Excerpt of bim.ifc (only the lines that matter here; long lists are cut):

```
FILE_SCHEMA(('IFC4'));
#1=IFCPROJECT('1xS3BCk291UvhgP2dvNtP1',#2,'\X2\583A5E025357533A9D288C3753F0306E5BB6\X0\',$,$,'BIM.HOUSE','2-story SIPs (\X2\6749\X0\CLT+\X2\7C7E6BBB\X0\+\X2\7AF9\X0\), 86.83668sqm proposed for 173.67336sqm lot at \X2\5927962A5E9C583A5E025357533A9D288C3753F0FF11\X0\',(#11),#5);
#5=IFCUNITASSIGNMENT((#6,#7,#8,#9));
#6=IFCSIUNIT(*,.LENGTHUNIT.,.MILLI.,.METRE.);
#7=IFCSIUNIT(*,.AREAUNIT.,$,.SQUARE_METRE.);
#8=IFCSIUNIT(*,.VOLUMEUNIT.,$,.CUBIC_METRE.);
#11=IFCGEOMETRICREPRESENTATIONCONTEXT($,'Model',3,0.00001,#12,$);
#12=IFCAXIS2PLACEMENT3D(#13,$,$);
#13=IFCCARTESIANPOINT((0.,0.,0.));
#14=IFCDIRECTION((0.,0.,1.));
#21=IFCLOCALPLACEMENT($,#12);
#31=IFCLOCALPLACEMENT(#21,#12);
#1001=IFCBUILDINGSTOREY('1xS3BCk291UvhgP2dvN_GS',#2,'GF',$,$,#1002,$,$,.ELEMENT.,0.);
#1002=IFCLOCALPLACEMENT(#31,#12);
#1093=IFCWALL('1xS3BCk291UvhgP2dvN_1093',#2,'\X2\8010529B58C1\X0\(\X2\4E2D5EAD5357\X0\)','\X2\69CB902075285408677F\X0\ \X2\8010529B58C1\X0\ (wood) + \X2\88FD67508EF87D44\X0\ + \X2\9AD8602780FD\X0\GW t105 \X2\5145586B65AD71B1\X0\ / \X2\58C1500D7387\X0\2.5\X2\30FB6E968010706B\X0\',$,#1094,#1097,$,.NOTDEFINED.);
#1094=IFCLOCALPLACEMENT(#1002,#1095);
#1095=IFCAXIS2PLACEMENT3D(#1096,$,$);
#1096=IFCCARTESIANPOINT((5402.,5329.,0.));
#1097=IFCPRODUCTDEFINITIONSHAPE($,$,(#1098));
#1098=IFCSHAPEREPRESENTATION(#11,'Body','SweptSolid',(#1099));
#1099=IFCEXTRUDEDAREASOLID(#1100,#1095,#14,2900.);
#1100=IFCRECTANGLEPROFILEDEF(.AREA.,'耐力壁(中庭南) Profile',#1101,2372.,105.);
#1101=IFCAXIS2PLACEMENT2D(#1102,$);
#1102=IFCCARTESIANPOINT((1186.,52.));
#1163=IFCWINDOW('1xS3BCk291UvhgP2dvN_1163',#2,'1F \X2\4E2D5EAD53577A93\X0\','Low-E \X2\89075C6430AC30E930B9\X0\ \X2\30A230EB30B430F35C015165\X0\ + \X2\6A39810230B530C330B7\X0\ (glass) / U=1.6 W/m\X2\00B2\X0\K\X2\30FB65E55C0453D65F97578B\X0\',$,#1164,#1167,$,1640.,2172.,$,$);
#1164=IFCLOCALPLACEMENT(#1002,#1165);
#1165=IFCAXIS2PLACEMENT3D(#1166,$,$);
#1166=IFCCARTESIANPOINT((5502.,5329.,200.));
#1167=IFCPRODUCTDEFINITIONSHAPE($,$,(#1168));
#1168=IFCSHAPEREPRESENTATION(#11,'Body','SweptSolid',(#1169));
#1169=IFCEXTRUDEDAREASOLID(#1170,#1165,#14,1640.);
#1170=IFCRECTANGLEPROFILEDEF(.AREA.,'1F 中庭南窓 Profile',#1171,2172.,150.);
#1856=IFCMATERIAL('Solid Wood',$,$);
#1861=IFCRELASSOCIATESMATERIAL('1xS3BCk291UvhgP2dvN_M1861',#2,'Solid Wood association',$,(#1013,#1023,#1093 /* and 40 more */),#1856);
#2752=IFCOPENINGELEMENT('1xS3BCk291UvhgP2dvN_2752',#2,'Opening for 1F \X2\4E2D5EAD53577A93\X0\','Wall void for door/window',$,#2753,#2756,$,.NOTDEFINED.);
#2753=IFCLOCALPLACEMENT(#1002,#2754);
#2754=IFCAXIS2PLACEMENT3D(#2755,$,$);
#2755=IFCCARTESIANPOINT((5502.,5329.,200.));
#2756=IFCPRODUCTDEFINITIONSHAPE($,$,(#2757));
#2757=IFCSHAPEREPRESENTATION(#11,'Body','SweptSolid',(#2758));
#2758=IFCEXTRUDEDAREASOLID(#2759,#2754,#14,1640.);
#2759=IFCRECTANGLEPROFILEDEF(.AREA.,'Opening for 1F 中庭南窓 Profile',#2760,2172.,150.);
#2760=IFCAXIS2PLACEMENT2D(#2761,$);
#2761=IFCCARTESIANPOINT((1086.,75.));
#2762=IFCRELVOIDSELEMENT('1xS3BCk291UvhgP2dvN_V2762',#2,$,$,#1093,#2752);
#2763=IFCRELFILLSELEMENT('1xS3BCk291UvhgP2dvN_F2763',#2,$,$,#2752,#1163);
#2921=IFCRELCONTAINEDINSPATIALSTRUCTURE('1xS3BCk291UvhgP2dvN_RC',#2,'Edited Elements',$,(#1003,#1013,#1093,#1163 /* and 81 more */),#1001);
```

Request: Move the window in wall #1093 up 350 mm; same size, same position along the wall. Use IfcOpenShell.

```python
import numpy as np
import ifcopenshell
import ifcopenshell.api.geometry
import ifcopenshell.util.placement
import ifcopenshell.util.unit

model = ifcopenshell.open("bim.ifc")
unit_scale = ifcopenshell.util.unit.calculate_unit_scale(model)

window = model.by_guid("1xS3BCk291UvhgP2dvN_1163")
opening = window.FillsVoids[0].RelatingOpeningElement
dz = 350.0

shift = np.array([0.0, 0.0, dz])
# The window is not placed relative to its opening, so move both.
for product in (opening, window):
    matrix = ifcopenshell.util.placement.get_local_placement(product.ObjectPlacement)
    matrix[:3, 3] += shift
    ifcopenshell.api.geometry.edit_object_placement(model, product=product, matrix=matrix, is_si=False)

print(f"moved by {dz * unit_scale:+.3f} m")

model.write("bim_edited.ifc")
```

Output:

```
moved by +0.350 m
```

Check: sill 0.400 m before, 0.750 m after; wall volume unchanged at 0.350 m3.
